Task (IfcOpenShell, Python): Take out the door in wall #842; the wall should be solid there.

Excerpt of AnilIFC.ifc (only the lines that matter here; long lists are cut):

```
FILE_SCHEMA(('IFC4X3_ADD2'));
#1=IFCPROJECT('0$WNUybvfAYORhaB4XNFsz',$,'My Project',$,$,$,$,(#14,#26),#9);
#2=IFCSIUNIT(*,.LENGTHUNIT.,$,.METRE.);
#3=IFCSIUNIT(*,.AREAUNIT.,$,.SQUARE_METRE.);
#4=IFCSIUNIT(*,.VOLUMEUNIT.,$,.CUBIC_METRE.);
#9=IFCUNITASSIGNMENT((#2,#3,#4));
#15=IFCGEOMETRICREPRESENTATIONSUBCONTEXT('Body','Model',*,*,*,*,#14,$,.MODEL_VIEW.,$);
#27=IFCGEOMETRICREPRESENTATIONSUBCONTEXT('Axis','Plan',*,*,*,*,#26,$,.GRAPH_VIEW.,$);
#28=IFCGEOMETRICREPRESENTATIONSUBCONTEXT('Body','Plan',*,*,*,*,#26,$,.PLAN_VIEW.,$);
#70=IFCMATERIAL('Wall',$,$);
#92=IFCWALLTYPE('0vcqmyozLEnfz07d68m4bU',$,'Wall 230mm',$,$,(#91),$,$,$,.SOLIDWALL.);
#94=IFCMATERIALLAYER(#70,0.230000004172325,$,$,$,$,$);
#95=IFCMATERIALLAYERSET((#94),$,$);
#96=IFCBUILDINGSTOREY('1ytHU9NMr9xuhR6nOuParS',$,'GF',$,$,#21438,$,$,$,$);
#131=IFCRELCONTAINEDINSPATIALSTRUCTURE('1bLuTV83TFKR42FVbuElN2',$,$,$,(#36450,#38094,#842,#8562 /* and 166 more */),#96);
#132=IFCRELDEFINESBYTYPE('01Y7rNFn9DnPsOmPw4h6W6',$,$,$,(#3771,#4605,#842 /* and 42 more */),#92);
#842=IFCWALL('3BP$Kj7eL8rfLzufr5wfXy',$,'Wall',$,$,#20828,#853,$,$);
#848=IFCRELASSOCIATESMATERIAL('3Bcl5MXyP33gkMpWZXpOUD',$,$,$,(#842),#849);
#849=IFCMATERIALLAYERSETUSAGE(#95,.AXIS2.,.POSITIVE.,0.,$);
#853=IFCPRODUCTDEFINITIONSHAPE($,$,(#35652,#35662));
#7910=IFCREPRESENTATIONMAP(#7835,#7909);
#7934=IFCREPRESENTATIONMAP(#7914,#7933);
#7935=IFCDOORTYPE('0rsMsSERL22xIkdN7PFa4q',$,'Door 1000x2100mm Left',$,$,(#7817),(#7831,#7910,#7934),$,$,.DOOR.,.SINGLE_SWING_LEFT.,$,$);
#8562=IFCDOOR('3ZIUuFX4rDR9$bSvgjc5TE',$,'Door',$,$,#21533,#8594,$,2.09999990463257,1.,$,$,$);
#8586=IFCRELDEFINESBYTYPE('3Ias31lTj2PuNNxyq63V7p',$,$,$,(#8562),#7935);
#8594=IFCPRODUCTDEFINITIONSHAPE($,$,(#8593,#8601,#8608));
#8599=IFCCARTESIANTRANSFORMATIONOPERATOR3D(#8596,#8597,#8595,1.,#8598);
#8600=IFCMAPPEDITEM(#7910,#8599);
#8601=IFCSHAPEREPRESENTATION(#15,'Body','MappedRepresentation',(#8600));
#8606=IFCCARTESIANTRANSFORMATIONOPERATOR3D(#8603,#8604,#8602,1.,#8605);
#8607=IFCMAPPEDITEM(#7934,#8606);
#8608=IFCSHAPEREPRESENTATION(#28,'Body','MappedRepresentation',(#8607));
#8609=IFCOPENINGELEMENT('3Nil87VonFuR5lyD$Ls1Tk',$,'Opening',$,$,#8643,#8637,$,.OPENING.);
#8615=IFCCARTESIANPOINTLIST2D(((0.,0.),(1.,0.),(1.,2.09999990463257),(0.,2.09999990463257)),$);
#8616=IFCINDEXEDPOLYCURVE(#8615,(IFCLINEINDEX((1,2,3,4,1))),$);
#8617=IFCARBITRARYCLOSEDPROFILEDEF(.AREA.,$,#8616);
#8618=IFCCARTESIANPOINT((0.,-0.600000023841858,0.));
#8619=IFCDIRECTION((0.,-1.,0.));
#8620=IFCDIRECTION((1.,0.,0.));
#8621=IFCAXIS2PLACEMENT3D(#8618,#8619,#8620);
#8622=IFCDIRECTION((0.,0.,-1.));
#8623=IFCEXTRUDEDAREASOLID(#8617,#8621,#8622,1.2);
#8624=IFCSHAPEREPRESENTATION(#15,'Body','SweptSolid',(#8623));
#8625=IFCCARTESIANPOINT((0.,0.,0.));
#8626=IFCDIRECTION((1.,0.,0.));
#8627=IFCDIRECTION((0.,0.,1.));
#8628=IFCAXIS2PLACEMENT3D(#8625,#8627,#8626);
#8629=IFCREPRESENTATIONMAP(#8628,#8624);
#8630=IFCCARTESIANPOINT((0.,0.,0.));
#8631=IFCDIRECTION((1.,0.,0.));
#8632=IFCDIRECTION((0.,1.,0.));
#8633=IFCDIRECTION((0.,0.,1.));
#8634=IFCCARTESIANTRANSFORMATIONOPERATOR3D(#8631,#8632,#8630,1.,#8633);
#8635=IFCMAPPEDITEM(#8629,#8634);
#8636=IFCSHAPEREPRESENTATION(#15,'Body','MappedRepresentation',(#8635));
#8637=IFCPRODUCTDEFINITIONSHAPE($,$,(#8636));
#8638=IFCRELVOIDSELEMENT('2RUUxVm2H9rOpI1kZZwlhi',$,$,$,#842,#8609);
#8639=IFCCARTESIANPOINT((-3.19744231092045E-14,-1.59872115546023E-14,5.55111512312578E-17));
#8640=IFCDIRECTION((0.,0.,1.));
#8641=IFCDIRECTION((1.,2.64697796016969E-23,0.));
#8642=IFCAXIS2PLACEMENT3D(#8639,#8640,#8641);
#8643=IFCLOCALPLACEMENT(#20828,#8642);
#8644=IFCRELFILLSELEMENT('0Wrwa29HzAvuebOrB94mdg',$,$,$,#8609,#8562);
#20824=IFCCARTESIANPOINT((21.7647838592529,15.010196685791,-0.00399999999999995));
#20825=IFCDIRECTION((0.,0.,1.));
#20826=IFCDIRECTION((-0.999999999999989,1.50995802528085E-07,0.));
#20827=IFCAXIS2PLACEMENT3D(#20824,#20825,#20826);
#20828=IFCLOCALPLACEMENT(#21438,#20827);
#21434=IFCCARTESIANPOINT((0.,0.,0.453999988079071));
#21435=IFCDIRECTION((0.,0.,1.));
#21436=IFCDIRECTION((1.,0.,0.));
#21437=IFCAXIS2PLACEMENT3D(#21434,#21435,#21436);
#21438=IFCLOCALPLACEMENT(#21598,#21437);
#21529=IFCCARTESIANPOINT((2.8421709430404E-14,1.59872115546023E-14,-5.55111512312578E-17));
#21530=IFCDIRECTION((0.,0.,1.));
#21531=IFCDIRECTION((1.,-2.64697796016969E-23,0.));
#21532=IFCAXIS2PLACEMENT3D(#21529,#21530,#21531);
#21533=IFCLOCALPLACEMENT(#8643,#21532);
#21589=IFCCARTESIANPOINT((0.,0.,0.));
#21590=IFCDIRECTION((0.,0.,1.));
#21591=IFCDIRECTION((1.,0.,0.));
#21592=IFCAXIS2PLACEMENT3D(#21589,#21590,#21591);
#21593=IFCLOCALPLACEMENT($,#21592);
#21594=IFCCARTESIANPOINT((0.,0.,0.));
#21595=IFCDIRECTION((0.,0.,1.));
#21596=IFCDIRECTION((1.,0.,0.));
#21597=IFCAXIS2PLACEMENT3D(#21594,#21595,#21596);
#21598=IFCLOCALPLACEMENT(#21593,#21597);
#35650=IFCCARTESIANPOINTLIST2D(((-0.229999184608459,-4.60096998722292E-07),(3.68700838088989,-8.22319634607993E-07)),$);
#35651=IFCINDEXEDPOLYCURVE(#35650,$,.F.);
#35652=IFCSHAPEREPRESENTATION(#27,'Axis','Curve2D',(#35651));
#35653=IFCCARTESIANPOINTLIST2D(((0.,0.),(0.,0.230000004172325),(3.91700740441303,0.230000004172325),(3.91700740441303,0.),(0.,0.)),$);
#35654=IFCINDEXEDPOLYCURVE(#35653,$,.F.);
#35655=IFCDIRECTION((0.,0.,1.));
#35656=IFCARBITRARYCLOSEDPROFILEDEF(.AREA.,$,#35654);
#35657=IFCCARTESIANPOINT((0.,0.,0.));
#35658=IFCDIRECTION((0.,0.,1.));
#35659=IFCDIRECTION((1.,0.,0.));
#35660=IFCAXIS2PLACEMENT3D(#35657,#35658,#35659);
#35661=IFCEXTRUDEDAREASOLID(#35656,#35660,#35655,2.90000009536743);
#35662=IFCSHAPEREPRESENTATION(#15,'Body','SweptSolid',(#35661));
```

```python
import ifcopenshell
import ifcopenshell.api.feature
import ifcopenshell.api.root
import ifcopenshell.geom
import ifcopenshell.util.shape

model = ifcopenshell.open("AnilIFC.ifc")
settings = ifcopenshell.geom.settings()


def volume(element):
    """Net volume in cubic metres, openings subtracted."""
    shape = ifcopenshell.geom.create_shape(settings, element)
    return ifcopenshell.util.shape.get_volume(shape.geometry)


door = model.by_guid("3ZIUuFX4rDR9$bSvgjc5TE")
opening = door.FillsVoids[0].RelatingOpeningElement
wall = opening.VoidsElements[0].RelatingBuildingElement
before = volume(wall)

ifcopenshell.api.root.remove_product(model, product=door)
ifcopenshell.api.feature.remove_feature(model, feature=opening)

after = volume(wall)

print(f"wall volume {before:.3f} -> {after:.3f} m3")

model.write("AnilIFC-out.ifc")
```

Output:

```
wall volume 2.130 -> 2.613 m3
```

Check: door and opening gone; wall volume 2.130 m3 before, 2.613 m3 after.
